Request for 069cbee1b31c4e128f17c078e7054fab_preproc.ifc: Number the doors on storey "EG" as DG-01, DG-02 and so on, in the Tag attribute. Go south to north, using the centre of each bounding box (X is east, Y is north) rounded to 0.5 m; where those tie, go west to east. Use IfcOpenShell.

First a look at what the model holds.

```python
import ifcopenshell
import ifcopenshell.util.element
import ifcopenshell.util.placement

model = ifcopenshell.open("069cbee1b31c4e128f17c078e7054fab_preproc.ifc")
print(model.schema)
storey = next(s for s in model.by_type("IfcBuildingStorey") if s.Name == "EG")
doors = [e for e in ifcopenshell.util.element.get_decomposition(storey) if e.is_a("IfcDoor")]
for e in sorted(doors, key=lambda e: e.id()):
    origin = ifcopenshell.util.placement.get_local_placement(e.ObjectPlacement)[:3, 3]
    print(e.id(), e.Tag, e.Name, origin.round(2) + 0.0, sep=" | ")
```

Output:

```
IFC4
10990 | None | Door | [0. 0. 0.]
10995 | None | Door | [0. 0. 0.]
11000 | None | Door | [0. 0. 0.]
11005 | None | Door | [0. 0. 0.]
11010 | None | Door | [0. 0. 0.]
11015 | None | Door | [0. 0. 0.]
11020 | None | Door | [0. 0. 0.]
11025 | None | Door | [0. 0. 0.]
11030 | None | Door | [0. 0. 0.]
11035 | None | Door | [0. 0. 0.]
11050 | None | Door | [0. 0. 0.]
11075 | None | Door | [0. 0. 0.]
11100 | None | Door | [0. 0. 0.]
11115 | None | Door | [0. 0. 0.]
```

```python
import ifcopenshell
import ifcopenshell.geom
import ifcopenshell.util.element
import ifcopenshell.util.shape

model = ifcopenshell.open("069cbee1b31c4e128f17c078e7054fab_preproc.ifc")
settings = ifcopenshell.geom.settings()
settings.set("use-world-coords", True)


def centre(element):
    shape = ifcopenshell.geom.create_shape(settings, element)
    return ifcopenshell.util.shape.get_bbox_centroid(shape.geometry)


storey = next(s for s in model.by_type("IfcBuildingStorey") if s.Name == "EG")
doors = [e for e in ifcopenshell.util.element.get_decomposition(storey) if e.is_a("IfcDoor")]

# Insertion points can sit at a corner or the storey origin, so sort by the geometry (in metres).
centres = {e: centre(e) for e in doors}
doors.sort(key=lambda e: (round(centres[e][1] / 0.5), centres[e][0]))

for i, e in enumerate(doors, start=1):
    number = f"DG-{i:02d}"
    e.Tag = number
    print(e.id(), number)

model.write("069cbee1b31c4e128f17c078e7054fab_preproc-out.ifc")
```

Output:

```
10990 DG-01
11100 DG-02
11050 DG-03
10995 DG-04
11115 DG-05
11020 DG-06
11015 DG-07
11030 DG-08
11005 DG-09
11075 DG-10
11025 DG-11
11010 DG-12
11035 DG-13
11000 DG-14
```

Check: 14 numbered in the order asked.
